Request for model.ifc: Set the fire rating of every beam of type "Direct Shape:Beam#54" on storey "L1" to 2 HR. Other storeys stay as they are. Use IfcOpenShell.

First a look at what the model holds.

```python
import ifcopenshell
import ifcopenshell.util.element

model = ifcopenshell.open("model.ifc")
print(model.schema)
storey = next(s for s in model.by_type("IfcBuildingStorey") if s.Name == "L1")
beams = [e for e in ifcopenshell.util.element.get_decomposition(storey) if e.is_a("IfcBeam")]
seen = {}
for e in beams:
    element_type = ifcopenshell.util.element.get_type(e)
    key = (element_type.Name if element_type != e and element_type else None, ifcopenshell.util.element.get_pset(e, "Pset_BeamCommon", "FireRating"))
    seen[key] = seen.get(key, 0) + 1
for (name, value), count in sorted(seen.items(), key=str):
    print(count, "x", name, "|", value)
```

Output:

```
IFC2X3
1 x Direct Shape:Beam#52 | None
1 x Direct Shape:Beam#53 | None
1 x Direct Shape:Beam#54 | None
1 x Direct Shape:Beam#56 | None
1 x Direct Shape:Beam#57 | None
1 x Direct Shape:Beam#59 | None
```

```python
import ifcopenshell
import ifcopenshell.api.pset
import ifcopenshell.util.element

model = ifcopenshell.open("model.ifc")

storey = next(s for s in model.by_type("IfcBuildingStorey") if s.Name == "L1")
beams = [e for e in ifcopenshell.util.element.get_decomposition(storey) if e.is_a("IfcBeam")]

count = 0
for e in beams:
    element_type = ifcopenshell.util.element.get_type(e)
    if element_type in (None, e) or element_type.Name != "Direct Shape:Beam#54":
        continue
    # add_pset returns the element's existing set when there is one.
    pset = ifcopenshell.api.pset.add_pset(model, product=e, name="Pset_BeamCommon")
    ifcopenshell.api.pset.edit_pset(model, pset=pset, properties={"FireRating": "2 HR"})
    count += 1

print(count, "beams updated")

model.write("model_rev.ifc")
```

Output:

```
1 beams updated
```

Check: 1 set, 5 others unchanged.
